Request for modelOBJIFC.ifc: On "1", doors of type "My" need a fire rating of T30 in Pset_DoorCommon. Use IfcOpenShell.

First a look at what the model holds.

```python
import ifcopenshell
import ifcopenshell.util.element

model = ifcopenshell.open("modelOBJIFC.ifc")
print(model.schema)
storey = next(s for s in model.by_type("IfcBuildingStorey") if s.Name == "1")
doors = [e for e in ifcopenshell.util.element.get_decomposition(storey) if e.is_a("IfcDoor")]
seen = {}
for e in doors:
    element_type = ifcopenshell.util.element.get_type(e)
    key = (element_type.Name if element_type != e and element_type else None, ifcopenshell.util.element.get_pset(e, "Pset_DoorCommon", "FireRating"))
    seen[key] = seen.get(key, 0) + 1
for (name, value), count in sorted(seen.items(), key=str):
    print(count, "x", name, "|", value)
```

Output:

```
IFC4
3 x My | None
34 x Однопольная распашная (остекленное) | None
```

```python
import ifcopenshell
import ifcopenshell.api.pset
import ifcopenshell.util.element

model = ifcopenshell.open("modelOBJIFC.ifc")

storey = next(s for s in model.by_type("IfcBuildingStorey") if s.Name == "1")
doors = [e for e in ifcopenshell.util.element.get_decomposition(storey) if e.is_a("IfcDoor")]

count = 0
for e in doors:
    element_type = ifcopenshell.util.element.get_type(e)
    if element_type in (None, e) or element_type.Name != "My":
        continue
    # add_pset returns the element's existing set when there is one.
    pset = ifcopenshell.api.pset.add_pset(model, product=e, name="Pset_DoorCommon")
    ifcopenshell.api.pset.edit_pset(model, pset=pset, properties={"FireRating": "T30"})
    count += 1

print(count, "doors updated")

model.write("modelOBJIFC_edited.ifc")
```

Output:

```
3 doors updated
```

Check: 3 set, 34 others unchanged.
